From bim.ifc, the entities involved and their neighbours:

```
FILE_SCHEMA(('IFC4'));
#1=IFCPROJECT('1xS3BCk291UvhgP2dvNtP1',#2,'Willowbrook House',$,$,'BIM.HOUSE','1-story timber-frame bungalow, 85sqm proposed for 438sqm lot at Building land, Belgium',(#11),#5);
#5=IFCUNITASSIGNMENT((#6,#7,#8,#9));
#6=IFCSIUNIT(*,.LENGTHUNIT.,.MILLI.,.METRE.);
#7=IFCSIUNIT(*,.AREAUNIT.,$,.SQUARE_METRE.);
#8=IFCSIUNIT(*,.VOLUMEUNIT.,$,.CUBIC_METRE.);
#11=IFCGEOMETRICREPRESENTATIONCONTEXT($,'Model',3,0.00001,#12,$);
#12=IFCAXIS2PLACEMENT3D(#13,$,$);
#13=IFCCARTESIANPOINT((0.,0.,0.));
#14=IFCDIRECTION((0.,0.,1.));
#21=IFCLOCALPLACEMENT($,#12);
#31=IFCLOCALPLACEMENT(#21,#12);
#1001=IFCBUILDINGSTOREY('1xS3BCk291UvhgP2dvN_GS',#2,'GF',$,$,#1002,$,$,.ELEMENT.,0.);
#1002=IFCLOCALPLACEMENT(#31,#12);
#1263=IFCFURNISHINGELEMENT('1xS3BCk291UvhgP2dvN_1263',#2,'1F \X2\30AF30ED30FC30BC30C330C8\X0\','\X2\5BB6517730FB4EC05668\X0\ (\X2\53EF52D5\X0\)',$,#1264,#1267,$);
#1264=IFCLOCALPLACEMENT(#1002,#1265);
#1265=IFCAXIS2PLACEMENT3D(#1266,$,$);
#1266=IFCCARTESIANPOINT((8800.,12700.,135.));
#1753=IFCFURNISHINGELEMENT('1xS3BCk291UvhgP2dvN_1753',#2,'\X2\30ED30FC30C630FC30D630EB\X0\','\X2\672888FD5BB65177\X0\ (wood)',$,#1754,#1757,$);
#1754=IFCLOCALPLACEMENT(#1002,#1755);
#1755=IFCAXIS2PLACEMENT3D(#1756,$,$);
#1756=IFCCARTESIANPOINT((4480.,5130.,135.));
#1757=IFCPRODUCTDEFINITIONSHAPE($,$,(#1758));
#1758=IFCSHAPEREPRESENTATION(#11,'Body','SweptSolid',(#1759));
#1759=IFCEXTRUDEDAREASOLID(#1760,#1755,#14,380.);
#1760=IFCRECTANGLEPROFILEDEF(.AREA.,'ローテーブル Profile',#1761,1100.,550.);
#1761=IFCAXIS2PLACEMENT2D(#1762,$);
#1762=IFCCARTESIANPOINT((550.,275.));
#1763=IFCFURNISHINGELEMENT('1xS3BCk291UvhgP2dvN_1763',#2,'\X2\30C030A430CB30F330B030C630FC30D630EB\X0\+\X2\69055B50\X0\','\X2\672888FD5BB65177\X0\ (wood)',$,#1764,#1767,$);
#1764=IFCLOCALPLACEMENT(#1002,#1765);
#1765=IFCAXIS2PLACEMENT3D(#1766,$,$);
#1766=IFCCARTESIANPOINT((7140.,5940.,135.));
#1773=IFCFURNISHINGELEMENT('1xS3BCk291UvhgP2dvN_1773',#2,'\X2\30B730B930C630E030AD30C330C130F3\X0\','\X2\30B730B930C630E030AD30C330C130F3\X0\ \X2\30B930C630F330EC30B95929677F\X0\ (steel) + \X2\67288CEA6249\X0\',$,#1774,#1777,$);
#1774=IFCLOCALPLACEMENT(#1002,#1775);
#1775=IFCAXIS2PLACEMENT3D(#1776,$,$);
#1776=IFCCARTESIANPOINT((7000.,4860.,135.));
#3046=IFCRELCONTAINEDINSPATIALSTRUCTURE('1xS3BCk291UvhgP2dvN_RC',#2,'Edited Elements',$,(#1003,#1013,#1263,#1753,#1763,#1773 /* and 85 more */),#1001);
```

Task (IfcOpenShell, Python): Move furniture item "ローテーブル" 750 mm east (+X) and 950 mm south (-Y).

```python
import ifcopenshell
import ifcopenshell.api.geometry
import ifcopenshell.util.placement

model = ifcopenshell.open("bim.ifc")

item = model.by_id(1753)
matrix = ifcopenshell.util.placement.get_local_placement(item.ObjectPlacement)
matrix[0, 3] += 750.0
matrix[1, 3] -= 950.0
ifcopenshell.api.geometry.edit_object_placement(model, product=item, matrix=matrix, is_si=False)

print(ifcopenshell.util.placement.get_local_placement(item.ObjectPlacement).round(3) + 0.0)

model.write("bim-out.ifc")
```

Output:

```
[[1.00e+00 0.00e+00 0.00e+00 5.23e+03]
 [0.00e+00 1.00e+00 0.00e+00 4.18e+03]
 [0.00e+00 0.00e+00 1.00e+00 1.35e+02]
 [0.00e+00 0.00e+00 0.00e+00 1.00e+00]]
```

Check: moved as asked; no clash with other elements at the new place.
